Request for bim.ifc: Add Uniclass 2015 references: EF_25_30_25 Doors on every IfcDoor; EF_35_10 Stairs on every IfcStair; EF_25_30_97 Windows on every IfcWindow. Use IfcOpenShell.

First a look at what the model holds.

```python
import ifcopenshell

model = ifcopenshell.open("bim.ifc")
print(model.schema)
print("classifications:", [c.Name for c in model.by_type("IfcClassification")])
for ifc_class in ("IfcDoor", "IfcRoof", "IfcStair", "IfcWall", "IfcWindow"):
    print(ifc_class, len(model.by_type(ifc_class)))
```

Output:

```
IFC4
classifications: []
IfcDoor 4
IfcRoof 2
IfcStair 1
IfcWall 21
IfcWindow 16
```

```python
import ifcopenshell
import ifcopenshell.api.classification

model = ifcopenshell.open("bim.ifc")

system = ifcopenshell.api.classification.add_classification(model, classification="Uniclass 2015")

codes = {
    "IfcDoor": ("EF_25_30_25", "Doors"),
    "IfcStair": ("EF_35_10", "Stairs"),
    "IfcWindow": ("EF_25_30_97", "Windows"),
}
for ifc_class, (code, name) in codes.items():
    products = model.by_type(ifc_class)
    ifcopenshell.api.classification.add_reference(
        model, products=products, classification=system, identification=code, name=name
    )
    print(code, len(products))

model.write("bim_edited.ifc")
```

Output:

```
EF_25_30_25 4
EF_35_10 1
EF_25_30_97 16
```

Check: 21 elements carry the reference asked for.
